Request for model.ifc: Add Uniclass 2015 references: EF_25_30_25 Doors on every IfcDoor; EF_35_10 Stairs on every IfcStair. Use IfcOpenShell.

First a look at what the model holds.

```python
import ifcopenshell

model = ifcopenshell.open("model.ifc")
print(model.schema)
print("classifications:", [c.Name for c in model.by_type("IfcClassification")])
for ifc_class in ("IfcDoor", "IfcRoof", "IfcStair", "IfcWall", "IfcWindow"):
    print(ifc_class, len(model.by_type(ifc_class)))
```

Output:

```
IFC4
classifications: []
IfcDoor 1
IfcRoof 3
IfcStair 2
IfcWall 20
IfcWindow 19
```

```python
import ifcopenshell
import ifcopenshell.api.classification

model = ifcopenshell.open("model.ifc")

system = ifcopenshell.api.classification.add_classification(model, classification="Uniclass 2015")

codes = {
    "IfcDoor": ("EF_25_30_25", "Doors"),
    "IfcStair": ("EF_35_10", "Stairs"),
}
for ifc_class, (code, name) in codes.items():
    products = model.by_type(ifc_class)
    ifcopenshell.api.classification.add_reference(
        model, products=products, classification=system, identification=code, name=name
    )
    print(code, len(products))

model.write("model_updated.ifc")
```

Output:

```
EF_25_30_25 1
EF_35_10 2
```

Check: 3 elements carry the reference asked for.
